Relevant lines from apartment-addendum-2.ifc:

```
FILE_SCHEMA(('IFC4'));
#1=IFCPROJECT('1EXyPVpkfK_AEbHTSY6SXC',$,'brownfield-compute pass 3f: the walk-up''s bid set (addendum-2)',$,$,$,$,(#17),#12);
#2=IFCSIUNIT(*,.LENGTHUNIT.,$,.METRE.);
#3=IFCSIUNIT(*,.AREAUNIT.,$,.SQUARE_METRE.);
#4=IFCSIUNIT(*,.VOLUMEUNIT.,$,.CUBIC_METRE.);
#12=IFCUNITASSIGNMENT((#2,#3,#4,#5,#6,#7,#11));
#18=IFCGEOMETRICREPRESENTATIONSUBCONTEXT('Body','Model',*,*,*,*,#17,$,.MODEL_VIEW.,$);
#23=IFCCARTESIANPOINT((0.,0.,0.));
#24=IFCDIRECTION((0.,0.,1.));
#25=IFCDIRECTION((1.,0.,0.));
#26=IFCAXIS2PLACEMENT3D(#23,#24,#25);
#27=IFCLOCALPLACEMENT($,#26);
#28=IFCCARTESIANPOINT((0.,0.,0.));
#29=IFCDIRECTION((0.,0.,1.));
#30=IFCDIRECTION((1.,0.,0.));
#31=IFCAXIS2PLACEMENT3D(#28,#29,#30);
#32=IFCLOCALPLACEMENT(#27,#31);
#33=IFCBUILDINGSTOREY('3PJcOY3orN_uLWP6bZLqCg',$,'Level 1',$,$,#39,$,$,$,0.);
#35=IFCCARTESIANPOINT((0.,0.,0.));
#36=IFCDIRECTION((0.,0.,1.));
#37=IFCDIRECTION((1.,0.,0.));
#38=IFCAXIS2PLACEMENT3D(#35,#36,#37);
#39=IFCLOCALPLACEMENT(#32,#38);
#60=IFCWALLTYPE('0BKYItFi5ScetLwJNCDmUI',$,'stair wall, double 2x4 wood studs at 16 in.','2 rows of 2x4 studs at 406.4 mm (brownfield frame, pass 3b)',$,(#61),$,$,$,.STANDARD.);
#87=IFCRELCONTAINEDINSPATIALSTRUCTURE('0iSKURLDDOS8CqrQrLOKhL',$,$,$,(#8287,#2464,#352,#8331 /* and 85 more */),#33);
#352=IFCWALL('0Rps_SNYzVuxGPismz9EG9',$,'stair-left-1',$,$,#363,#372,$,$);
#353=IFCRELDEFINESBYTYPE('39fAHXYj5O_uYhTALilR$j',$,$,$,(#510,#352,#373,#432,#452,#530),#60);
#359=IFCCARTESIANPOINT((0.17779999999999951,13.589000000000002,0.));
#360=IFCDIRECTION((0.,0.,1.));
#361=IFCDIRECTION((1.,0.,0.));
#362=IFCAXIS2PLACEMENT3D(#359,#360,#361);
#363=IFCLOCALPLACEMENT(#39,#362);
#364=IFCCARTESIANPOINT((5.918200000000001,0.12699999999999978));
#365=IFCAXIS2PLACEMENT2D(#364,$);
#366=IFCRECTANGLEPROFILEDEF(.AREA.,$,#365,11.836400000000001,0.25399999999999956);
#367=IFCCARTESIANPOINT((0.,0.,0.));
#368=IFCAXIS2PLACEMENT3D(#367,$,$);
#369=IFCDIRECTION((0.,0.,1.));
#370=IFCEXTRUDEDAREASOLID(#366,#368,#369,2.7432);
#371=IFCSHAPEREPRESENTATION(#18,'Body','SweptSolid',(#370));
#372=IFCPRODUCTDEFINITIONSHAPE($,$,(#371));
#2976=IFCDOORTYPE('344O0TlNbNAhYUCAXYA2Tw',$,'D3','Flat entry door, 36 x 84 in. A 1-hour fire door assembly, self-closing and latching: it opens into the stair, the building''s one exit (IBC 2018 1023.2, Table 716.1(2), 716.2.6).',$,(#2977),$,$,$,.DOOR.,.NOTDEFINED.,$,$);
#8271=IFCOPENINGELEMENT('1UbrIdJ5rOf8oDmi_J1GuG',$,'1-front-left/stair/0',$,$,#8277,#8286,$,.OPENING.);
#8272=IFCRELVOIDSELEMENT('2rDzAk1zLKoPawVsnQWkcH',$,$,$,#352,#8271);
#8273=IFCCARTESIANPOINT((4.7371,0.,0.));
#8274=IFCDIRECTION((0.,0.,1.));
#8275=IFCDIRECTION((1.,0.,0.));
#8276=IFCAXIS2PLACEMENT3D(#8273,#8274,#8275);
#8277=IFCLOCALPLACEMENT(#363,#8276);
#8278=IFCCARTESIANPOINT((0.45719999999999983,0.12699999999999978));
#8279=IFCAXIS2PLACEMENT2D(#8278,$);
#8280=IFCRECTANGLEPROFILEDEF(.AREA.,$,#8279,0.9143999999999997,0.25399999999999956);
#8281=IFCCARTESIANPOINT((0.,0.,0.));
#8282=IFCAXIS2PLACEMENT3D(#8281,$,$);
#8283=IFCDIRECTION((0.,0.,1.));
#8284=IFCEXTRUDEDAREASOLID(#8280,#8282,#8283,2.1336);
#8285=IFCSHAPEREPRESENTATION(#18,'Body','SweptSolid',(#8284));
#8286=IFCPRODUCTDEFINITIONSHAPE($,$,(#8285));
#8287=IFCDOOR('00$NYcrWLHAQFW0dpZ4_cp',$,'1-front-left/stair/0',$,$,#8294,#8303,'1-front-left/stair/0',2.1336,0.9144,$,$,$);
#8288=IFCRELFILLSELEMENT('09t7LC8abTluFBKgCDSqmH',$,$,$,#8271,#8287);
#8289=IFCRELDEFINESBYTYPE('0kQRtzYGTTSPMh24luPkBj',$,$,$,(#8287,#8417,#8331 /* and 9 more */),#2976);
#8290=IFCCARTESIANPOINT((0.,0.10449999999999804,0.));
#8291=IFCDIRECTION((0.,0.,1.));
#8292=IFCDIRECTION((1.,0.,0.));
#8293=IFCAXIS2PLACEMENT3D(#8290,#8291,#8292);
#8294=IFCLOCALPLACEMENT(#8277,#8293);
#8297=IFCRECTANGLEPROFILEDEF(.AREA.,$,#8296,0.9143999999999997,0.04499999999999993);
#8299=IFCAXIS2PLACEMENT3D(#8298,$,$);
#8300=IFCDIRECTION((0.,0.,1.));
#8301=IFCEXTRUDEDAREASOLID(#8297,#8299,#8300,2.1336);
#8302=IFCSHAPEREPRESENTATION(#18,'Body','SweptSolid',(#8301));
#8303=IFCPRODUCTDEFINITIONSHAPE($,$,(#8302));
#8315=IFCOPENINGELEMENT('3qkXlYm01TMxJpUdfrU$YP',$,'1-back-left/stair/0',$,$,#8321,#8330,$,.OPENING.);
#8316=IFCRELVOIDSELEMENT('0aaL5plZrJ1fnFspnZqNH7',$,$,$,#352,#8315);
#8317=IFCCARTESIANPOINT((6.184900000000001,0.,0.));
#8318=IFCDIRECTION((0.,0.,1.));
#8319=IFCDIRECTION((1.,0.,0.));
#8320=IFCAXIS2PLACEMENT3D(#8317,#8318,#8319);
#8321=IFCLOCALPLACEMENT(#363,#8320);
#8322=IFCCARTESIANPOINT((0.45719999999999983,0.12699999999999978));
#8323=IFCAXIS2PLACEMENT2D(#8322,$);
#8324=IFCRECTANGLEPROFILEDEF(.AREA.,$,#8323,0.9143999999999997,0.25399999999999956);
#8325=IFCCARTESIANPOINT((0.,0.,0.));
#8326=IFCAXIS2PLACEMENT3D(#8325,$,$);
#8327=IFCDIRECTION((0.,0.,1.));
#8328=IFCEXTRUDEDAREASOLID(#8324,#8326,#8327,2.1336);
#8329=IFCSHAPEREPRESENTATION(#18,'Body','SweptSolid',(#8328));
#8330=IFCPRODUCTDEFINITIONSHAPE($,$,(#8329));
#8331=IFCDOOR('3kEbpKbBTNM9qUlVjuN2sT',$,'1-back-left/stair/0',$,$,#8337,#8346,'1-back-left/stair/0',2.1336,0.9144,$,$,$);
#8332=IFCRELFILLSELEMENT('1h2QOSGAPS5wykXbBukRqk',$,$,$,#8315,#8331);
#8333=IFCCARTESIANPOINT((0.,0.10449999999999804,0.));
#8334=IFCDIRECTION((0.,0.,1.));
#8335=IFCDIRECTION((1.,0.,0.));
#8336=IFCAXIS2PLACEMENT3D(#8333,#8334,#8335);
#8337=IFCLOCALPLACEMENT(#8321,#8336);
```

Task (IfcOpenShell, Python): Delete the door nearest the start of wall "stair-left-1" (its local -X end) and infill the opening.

```python
import ifcopenshell
import ifcopenshell.api.feature
import ifcopenshell.api.root
import ifcopenshell.geom
import ifcopenshell.util.shape

model = ifcopenshell.open("apartment-addendum-2.ifc")
settings = ifcopenshell.geom.settings()


def volume(element):
    """Net volume in cubic metres, openings subtracted."""
    shape = ifcopenshell.geom.create_shape(settings, element)
    return ifcopenshell.util.shape.get_volume(shape.geometry)


door = model.by_guid("00$NYcrWLHAQFW0dpZ4_cp")
opening = door.FillsVoids[0].RelatingOpeningElement
wall = opening.VoidsElements[0].RelatingBuildingElement
before = volume(wall)

ifcopenshell.api.root.remove_product(model, product=door)
ifcopenshell.api.feature.remove_feature(model, feature=opening)

after = volume(wall)

print(f"wall volume {before:.3f} -> {after:.3f} m3")

model.write("apartment-addendum-2_v2.ifc")
```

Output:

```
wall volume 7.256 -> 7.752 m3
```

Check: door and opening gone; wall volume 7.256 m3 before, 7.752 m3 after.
